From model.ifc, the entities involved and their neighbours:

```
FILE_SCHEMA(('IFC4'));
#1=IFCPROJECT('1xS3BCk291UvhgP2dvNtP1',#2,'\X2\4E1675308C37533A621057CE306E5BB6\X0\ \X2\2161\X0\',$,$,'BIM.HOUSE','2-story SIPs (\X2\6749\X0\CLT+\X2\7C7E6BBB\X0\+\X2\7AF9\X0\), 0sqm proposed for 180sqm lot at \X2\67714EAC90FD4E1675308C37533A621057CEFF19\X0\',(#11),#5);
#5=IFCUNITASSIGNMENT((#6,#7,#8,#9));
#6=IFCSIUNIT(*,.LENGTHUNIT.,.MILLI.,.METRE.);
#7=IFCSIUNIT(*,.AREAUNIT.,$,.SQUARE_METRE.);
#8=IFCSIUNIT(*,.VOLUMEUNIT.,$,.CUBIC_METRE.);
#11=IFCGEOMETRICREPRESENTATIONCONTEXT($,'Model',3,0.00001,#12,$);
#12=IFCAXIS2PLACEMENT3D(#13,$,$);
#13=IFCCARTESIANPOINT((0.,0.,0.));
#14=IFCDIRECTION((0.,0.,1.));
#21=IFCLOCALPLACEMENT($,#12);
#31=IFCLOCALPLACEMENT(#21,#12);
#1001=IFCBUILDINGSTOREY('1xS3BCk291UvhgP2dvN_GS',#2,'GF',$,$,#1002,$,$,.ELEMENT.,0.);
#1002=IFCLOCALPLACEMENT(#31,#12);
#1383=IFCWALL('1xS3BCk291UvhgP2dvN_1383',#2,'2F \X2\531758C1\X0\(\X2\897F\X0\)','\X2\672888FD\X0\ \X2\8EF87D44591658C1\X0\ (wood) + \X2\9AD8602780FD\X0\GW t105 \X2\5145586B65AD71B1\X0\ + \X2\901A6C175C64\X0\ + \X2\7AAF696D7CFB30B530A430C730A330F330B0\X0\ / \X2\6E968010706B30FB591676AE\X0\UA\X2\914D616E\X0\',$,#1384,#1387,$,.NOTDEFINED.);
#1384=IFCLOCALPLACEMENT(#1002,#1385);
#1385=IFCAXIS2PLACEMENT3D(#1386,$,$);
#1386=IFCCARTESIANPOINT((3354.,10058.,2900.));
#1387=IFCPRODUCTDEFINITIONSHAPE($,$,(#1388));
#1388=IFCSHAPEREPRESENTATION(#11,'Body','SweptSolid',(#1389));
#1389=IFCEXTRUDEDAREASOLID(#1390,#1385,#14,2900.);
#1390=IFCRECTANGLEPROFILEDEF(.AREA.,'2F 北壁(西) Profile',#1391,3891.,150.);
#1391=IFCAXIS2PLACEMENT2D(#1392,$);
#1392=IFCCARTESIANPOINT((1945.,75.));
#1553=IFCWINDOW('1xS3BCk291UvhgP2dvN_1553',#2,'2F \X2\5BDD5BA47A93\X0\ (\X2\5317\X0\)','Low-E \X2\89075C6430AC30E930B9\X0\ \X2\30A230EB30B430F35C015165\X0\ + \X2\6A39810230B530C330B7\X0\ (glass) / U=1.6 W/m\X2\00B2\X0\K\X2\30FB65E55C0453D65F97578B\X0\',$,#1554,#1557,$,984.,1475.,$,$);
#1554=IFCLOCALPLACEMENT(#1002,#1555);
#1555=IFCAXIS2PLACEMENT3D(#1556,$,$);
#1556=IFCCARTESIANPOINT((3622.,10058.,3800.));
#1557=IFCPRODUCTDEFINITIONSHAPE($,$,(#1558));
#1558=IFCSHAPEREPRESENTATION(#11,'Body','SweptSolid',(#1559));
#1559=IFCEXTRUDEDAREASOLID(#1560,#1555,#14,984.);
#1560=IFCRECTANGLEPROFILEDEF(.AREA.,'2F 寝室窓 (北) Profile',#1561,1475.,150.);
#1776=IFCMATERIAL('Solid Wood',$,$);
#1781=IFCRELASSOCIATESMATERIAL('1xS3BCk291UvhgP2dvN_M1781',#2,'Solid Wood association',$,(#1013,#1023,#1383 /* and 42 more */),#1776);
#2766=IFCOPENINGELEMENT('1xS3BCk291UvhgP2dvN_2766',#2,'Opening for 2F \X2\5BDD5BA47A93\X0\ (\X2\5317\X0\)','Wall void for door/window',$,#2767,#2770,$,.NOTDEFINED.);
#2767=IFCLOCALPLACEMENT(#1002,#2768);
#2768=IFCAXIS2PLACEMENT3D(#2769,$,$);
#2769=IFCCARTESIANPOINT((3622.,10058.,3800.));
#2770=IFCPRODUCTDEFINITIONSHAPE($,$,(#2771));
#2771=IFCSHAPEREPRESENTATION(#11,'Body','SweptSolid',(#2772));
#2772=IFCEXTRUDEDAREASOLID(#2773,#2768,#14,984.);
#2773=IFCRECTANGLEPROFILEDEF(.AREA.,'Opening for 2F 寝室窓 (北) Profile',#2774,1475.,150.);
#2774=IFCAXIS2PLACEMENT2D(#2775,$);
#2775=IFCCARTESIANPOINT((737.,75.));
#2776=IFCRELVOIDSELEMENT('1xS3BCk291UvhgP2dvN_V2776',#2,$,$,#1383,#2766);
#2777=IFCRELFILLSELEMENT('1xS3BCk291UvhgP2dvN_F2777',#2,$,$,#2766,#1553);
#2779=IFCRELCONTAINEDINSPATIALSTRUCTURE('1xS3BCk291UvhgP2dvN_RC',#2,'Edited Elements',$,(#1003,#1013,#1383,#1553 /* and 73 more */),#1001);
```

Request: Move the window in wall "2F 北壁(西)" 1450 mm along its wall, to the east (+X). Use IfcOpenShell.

```python
import ifcopenshell
import ifcopenshell.api.geometry
import ifcopenshell.util.placement
import ifcopenshell.util.unit

model = ifcopenshell.open("model.ifc")
unit_scale = ifcopenshell.util.unit.calculate_unit_scale(model)

window = model.by_id(1553)
opening = window.FillsVoids[0].RelatingOpeningElement
wall = opening.VoidsElements[0].RelatingBuildingElement

wall_matrix = ifcopenshell.util.placement.get_local_placement(wall.ObjectPlacement)
shift = wall_matrix[:3, 0] * 1.45 / unit_scale
before = ifcopenshell.util.placement.get_local_placement(window.ObjectPlacement)[:3, 3].copy()

# The window is not placed relative to its opening, so move both.
for product in (opening, window):
    matrix = ifcopenshell.util.placement.get_local_placement(product.ObjectPlacement)
    matrix[:3, 3] += shift
    ifcopenshell.api.geometry.edit_object_placement(model, product=product, matrix=matrix, is_si=False)

after = ifcopenshell.util.placement.get_local_placement(window.ObjectPlacement)[:3, 3]
print("window moved by", (after - before).round(3) + 0.0)

model.write("model_v2.ifc")
```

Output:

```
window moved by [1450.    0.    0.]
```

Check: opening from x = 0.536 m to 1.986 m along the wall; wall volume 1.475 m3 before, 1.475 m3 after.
